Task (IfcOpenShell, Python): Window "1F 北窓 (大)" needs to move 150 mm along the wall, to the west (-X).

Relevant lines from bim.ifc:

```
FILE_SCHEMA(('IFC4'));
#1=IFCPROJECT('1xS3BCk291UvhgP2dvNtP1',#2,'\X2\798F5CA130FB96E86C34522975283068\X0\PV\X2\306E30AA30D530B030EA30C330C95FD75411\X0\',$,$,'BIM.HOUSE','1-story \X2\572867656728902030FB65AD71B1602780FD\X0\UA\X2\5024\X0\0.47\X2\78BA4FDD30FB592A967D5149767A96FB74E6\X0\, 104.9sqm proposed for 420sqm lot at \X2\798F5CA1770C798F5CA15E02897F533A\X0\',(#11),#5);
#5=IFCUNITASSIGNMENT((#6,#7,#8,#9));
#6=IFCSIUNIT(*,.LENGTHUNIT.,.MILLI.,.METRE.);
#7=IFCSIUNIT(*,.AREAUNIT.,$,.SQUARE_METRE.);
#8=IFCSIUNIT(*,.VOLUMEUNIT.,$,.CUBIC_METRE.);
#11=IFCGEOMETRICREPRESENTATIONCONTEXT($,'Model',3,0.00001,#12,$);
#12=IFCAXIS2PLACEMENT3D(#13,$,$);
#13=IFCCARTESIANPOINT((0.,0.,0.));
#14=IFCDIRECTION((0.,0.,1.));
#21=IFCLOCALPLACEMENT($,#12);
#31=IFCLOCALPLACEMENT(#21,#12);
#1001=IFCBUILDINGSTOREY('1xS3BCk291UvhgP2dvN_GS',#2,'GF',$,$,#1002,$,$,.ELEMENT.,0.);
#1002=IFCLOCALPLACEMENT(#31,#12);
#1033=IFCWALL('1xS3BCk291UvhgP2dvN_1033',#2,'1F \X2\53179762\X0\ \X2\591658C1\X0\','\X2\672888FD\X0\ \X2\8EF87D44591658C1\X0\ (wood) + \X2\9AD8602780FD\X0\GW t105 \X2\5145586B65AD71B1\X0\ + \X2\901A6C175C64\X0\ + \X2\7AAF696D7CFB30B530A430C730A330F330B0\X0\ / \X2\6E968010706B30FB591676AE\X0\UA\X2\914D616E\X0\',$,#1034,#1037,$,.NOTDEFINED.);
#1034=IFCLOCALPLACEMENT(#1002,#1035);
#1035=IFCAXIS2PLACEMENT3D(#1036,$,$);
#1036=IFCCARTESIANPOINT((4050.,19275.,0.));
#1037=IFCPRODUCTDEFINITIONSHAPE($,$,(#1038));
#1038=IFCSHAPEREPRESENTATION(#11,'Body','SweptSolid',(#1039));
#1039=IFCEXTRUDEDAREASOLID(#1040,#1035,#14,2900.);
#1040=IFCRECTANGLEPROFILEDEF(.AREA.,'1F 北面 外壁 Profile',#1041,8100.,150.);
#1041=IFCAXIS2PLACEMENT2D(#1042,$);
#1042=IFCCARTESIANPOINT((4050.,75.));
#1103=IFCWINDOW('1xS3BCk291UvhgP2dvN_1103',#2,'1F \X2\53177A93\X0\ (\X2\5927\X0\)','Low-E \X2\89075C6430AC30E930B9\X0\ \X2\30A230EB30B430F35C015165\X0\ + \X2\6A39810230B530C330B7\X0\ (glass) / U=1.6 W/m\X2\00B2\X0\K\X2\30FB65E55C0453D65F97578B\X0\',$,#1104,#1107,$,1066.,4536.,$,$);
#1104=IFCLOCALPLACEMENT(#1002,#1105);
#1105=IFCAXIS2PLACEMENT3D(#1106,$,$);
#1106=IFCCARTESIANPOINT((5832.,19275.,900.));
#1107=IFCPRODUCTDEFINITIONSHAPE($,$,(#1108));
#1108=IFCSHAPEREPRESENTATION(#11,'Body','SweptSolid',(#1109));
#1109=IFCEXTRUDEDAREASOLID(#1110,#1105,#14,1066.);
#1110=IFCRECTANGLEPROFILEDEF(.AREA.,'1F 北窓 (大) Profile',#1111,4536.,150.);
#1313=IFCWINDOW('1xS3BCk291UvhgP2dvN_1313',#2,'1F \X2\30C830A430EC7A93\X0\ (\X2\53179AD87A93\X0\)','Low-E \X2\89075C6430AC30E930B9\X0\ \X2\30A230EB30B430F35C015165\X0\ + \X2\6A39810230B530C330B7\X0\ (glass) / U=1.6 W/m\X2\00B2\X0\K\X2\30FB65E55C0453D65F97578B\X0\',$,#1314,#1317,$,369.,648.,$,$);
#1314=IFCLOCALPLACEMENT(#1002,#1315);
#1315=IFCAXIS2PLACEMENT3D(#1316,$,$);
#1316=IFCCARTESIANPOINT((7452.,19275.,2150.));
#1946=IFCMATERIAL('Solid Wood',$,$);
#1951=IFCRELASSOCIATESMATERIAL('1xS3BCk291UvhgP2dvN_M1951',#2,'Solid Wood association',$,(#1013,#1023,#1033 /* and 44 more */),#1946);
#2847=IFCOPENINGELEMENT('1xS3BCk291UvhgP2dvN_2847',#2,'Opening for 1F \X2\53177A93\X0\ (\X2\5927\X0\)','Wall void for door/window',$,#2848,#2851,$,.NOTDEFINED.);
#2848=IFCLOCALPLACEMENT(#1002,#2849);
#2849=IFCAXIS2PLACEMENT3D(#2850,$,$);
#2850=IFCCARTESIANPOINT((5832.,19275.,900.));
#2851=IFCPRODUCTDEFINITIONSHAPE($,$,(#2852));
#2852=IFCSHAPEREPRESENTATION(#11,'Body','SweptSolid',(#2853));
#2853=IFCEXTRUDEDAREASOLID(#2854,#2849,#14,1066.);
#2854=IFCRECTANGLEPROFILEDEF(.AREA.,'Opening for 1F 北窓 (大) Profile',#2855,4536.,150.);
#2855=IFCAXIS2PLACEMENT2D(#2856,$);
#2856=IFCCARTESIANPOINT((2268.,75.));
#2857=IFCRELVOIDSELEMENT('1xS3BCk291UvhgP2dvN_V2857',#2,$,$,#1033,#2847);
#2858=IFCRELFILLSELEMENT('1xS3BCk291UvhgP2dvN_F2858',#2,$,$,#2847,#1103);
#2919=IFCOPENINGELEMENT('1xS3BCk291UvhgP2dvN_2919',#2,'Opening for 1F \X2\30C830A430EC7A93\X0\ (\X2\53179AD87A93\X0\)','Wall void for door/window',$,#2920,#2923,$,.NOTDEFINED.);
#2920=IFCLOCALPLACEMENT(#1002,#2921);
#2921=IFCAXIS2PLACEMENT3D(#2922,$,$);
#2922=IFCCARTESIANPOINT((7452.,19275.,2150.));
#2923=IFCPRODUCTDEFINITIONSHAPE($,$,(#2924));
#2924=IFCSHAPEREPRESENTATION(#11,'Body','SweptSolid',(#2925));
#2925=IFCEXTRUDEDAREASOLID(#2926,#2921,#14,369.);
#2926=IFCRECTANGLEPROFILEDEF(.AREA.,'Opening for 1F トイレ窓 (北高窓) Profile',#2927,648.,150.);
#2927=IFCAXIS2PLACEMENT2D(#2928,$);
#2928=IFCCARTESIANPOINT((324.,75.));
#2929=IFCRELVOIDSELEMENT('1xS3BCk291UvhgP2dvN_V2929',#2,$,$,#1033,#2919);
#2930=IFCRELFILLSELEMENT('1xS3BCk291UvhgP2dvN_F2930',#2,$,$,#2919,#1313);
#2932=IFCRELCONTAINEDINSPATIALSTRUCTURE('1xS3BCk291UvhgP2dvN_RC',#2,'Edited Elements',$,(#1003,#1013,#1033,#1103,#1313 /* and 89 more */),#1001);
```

```python
import ifcopenshell
import ifcopenshell.api.geometry
import ifcopenshell.util.placement
import ifcopenshell.util.unit

model = ifcopenshell.open("bim.ifc")
unit_scale = ifcopenshell.util.unit.calculate_unit_scale(model)

window = model.by_id(1103)
opening = window.FillsVoids[0].RelatingOpeningElement
wall = opening.VoidsElements[0].RelatingBuildingElement

wall_matrix = ifcopenshell.util.placement.get_local_placement(wall.ObjectPlacement)
shift = wall_matrix[:3, 0] * -0.15 / unit_scale
before = ifcopenshell.util.placement.get_local_placement(window.ObjectPlacement)[:3, 3].copy()

# The window is not placed relative to its opening, so move both.
for product in (opening, window):
    matrix = ifcopenshell.util.placement.get_local_placement(product.ObjectPlacement)
    matrix[:3, 3] += shift
    ifcopenshell.api.geometry.edit_object_placement(model, product=product, matrix=matrix, is_si=False)

after = ifcopenshell.util.placement.get_local_placement(window.ObjectPlacement)[:3, 3]
print("window moved by", (after - before).round(3) + 0.0)

model.write("bim_edited.ifc")
```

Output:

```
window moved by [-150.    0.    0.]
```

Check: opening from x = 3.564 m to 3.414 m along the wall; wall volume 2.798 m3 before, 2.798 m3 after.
